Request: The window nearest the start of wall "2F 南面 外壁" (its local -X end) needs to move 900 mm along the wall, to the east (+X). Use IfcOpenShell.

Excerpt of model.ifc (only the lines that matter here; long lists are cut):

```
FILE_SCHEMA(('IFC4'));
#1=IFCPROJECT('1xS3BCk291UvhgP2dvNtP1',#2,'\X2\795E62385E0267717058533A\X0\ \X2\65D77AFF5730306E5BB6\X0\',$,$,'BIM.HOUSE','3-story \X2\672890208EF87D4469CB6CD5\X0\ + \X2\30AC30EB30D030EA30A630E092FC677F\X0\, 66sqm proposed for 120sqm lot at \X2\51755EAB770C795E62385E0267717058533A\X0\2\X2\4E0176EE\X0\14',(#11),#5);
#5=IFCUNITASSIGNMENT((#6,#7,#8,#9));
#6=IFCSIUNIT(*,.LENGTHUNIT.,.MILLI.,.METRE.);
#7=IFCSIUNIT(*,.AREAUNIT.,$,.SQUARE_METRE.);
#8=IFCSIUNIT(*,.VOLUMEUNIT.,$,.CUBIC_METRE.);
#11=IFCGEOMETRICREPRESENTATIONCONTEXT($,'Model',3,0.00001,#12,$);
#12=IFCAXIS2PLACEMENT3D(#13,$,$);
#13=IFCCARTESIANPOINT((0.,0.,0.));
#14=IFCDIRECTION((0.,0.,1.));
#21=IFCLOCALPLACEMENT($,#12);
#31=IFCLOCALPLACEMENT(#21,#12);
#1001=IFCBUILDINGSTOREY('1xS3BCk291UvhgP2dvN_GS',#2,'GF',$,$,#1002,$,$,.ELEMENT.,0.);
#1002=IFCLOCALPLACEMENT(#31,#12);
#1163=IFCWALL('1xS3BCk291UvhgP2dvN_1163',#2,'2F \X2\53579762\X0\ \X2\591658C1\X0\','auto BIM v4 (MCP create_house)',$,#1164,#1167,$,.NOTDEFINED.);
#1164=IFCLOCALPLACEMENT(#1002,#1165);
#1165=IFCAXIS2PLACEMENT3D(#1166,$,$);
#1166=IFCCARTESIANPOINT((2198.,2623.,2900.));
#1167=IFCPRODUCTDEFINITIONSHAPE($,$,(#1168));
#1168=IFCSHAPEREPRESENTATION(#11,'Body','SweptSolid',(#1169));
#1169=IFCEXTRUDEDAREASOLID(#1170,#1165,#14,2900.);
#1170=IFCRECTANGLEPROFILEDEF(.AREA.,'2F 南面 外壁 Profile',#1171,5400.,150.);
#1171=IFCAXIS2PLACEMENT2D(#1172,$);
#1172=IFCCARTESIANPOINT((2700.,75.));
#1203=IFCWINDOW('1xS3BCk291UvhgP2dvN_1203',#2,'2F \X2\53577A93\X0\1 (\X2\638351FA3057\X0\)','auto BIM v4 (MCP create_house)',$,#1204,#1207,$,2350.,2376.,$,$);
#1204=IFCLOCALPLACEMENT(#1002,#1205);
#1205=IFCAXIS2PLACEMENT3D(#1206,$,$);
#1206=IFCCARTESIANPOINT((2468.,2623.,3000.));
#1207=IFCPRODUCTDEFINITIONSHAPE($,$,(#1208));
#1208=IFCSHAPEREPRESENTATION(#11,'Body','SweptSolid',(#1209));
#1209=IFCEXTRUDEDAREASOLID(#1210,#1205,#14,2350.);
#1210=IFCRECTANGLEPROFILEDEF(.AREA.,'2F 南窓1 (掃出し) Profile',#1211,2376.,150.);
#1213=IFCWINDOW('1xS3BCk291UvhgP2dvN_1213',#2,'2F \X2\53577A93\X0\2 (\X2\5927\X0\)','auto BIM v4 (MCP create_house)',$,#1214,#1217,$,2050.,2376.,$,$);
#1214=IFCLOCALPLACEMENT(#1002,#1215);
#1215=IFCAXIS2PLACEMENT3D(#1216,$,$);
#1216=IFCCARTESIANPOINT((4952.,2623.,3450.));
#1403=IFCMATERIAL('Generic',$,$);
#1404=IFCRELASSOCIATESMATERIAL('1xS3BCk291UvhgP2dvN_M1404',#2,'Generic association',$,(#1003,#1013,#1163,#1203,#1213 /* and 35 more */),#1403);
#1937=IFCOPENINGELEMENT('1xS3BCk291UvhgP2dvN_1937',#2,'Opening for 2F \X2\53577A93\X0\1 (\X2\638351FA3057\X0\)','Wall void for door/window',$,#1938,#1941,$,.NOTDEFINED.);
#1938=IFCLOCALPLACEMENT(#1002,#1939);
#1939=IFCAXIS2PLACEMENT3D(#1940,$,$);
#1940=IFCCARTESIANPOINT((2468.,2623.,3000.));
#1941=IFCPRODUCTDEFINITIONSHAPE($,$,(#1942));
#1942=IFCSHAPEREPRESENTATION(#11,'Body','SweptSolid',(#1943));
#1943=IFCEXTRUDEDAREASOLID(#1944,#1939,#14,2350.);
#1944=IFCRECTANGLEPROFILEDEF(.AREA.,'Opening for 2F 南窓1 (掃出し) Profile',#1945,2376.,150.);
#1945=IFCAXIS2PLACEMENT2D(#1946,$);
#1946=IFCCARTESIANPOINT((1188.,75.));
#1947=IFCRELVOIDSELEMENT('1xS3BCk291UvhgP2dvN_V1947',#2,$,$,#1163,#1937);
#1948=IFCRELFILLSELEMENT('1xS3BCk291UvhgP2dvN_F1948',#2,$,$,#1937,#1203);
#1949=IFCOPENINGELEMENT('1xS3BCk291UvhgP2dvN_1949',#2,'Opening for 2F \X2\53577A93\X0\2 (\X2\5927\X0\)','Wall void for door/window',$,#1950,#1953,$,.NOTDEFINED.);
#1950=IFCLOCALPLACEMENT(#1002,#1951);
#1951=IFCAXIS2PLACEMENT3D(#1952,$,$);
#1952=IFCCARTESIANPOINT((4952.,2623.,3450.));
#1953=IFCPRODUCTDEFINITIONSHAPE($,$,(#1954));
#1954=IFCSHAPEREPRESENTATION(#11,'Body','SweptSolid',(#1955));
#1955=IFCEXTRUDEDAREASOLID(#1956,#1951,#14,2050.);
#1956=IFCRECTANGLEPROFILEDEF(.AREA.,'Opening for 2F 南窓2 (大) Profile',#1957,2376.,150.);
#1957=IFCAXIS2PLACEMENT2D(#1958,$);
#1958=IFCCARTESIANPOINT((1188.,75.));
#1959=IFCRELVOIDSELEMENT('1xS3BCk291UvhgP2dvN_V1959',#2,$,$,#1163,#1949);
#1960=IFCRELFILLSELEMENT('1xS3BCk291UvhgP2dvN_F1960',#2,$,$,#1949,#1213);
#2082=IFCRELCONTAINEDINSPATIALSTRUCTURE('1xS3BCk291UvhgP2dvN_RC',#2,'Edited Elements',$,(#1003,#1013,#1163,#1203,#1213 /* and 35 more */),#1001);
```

```python
import ifcopenshell
import ifcopenshell.api.geometry
import ifcopenshell.util.placement
import ifcopenshell.util.unit

model = ifcopenshell.open("model.ifc")
unit_scale = ifcopenshell.util.unit.calculate_unit_scale(model)

window = model.by_guid("1xS3BCk291UvhgP2dvN_1203")
opening = window.FillsVoids[0].RelatingOpeningElement
wall = opening.VoidsElements[0].RelatingBuildingElement

wall_matrix = ifcopenshell.util.placement.get_local_placement(wall.ObjectPlacement)
shift = wall_matrix[:3, 0] * 0.9 / unit_scale
before = ifcopenshell.util.placement.get_local_placement(window.ObjectPlacement)[:3, 3].copy()

# The window is not placed relative to its opening, so move both.
for product in (opening, window):
    matrix = ifcopenshell.util.placement.get_local_placement(product.ObjectPlacement)
    matrix[:3, 3] += shift
    ifcopenshell.api.geometry.edit_object_placement(model, product=product, matrix=matrix, is_si=False)

after = ifcopenshell.util.placement.get_local_placement(window.ObjectPlacement)[:3, 3]
print("window moved by", (after - before).round(3) + 0.0)

model.write("model_v2.ifc")
```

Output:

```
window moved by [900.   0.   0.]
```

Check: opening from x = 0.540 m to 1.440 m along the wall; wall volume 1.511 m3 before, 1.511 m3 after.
